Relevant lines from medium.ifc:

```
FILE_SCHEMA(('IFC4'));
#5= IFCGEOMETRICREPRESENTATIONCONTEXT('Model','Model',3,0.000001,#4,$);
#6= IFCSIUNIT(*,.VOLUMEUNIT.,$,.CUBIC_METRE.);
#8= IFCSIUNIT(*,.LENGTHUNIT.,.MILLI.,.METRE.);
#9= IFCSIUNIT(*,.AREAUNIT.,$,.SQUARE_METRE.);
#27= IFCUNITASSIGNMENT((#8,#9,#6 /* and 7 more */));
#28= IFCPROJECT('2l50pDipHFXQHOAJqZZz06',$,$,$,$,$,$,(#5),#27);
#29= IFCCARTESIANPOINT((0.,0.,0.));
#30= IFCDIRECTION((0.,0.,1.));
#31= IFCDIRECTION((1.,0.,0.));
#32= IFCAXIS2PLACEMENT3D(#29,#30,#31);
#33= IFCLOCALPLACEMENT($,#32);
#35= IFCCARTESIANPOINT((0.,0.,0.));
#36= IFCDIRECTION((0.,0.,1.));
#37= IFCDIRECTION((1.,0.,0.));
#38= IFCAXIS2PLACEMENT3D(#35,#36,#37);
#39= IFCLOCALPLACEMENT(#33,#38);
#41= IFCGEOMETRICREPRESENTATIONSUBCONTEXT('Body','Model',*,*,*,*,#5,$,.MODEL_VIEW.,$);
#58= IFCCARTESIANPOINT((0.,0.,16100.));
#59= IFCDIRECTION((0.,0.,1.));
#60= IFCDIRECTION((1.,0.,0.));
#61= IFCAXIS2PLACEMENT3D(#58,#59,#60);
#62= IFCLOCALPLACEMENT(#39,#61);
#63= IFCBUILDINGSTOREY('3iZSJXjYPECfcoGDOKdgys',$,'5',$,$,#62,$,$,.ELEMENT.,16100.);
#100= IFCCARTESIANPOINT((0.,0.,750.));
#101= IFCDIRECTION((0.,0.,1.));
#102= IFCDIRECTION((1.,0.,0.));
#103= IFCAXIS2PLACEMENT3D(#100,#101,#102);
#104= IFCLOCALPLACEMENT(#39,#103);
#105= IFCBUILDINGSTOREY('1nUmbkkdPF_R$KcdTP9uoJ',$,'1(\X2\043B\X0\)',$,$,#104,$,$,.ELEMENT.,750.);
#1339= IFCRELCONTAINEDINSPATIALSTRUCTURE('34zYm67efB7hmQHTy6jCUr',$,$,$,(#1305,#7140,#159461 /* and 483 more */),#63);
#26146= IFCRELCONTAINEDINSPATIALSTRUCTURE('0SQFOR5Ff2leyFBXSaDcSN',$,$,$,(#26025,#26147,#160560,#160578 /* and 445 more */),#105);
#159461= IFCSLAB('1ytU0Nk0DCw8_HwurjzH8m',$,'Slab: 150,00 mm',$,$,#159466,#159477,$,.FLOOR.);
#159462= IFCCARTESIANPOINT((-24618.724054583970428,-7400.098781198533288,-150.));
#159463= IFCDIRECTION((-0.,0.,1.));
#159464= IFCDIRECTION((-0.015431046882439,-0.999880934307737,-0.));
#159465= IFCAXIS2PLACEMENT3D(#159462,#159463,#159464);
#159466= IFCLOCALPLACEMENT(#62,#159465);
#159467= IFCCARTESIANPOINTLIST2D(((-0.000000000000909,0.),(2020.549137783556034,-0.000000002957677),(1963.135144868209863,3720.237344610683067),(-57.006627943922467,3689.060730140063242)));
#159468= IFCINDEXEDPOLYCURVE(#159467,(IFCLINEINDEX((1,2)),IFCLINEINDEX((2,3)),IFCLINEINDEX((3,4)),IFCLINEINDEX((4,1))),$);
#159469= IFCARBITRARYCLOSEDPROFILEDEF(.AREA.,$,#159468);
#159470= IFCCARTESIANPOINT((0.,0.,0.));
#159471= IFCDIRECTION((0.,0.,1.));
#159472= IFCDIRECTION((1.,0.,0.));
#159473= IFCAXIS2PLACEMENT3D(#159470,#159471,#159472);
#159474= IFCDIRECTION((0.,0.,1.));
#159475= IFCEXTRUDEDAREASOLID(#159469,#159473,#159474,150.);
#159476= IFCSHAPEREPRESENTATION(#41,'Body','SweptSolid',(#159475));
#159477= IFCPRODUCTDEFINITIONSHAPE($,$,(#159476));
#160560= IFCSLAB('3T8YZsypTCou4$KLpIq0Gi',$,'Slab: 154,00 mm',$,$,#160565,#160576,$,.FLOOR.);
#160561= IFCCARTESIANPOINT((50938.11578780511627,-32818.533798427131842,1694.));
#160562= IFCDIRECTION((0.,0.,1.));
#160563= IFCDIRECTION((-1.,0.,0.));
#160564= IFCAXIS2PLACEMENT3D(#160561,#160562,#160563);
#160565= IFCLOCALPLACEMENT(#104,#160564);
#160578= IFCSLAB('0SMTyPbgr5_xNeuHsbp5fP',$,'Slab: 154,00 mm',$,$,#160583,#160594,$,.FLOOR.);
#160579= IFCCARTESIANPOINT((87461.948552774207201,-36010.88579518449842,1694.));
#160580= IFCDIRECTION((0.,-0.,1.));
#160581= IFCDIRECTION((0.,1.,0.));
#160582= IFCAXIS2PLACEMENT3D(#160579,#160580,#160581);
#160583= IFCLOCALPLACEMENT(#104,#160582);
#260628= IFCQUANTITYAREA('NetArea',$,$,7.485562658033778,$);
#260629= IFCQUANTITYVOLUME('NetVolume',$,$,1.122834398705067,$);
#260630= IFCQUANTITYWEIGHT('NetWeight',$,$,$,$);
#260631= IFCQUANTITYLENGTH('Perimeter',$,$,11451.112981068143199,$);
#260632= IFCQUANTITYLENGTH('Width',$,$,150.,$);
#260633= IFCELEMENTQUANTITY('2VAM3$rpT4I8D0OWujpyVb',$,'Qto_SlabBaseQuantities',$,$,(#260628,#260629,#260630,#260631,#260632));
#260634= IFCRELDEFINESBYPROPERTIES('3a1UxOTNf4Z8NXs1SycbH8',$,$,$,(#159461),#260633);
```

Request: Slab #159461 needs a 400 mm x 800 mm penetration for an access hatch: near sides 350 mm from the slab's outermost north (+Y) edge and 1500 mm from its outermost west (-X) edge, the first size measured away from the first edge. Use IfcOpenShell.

```python
import numpy as np
import ifcopenshell
import ifcopenshell.api.feature
import ifcopenshell.api.geometry
import ifcopenshell.api.pset
import ifcopenshell.api.root
import ifcopenshell.geom
import ifcopenshell.util.element
import ifcopenshell.util.placement
import ifcopenshell.util.representation
import ifcopenshell.util.shape
import ifcopenshell.util.unit

model = ifcopenshell.open("medium.ifc")
unit_scale = ifcopenshell.util.unit.calculate_unit_scale(model)
area_scale = ifcopenshell.util.unit.calculate_unit_scale(model, "AREAUNIT")
volume_scale = ifcopenshell.util.unit.calculate_unit_scale(model, "VOLUMEUNIT")
settings = ifcopenshell.geom.settings()


def volume(element):
    """Net volume in cubic metres, openings subtracted."""
    shape = ifcopenshell.geom.create_shape(settings, element)
    return ifcopenshell.util.shape.get_volume(shape.geometry)


slab = model.by_guid("1ytU0Nk0DCw8_HwurjzH8m")
before = volume(slab)

# Extent in the slab's own axes, in metres. The edges named are its -X and -Y sides.
slab_shape = ifcopenshell.geom.create_shape(settings, slab)
vertices = ifcopenshell.util.shape.get_vertices(slab_shape.geometry)
x_min, y_min, bottom = vertices.min(axis=0)
top = vertices[:, 2].max()

opening = ifcopenshell.api.root.create_entity(model, ifc_class="IfcOpeningElement", name="Access hatch opening", predefined_type="OPENING")
context = ifcopenshell.util.representation.get_context(model, "Model", "Body", "MODEL_VIEW")
width, depth = 0.4, 0.8
outline = [(0.0, 0.0), (width, 0.0), (width, depth), (0.0, depth), (0.0, 0.0)]
# Overshoot both faces by 50 mm so the cut is clean.
shape = ifcopenshell.api.geometry.add_slab_representation(
    model, context=context, depth=top - bottom + 0.1, polyline=outline
)
ifcopenshell.api.geometry.assign_representation(model, product=opening, representation=shape)

matrix = ifcopenshell.util.placement.get_local_placement(slab.ObjectPlacement)
matrix[:, 3] = matrix @ np.append(np.array([x_min + 0.35, y_min + 1.5, bottom - 0.05]) / unit_scale, 1.0)
ifcopenshell.api.geometry.edit_object_placement(model, product=opening, matrix=matrix, is_si=False)
ifcopenshell.api.feature.add_feature(model, feature=opening, element=slab)

after = volume(slab)

# Update the slab's stored quantities.
qto = model.by_id(ifcopenshell.util.element.get_pset(slab, "Qto_SlabBaseQuantities", should_inherit=False)["id"])
ifcopenshell.api.pset.edit_qto(model, qto=qto, properties={
    "NetArea": after / (top - bottom) / area_scale,
    "NetVolume": after / volume_scale,
})

print(f"slab volume {before:.3f} -> {after:.3f} m3")

model.write("medium_rev.ifc")
```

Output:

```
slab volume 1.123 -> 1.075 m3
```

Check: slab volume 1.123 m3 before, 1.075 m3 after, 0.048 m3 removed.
